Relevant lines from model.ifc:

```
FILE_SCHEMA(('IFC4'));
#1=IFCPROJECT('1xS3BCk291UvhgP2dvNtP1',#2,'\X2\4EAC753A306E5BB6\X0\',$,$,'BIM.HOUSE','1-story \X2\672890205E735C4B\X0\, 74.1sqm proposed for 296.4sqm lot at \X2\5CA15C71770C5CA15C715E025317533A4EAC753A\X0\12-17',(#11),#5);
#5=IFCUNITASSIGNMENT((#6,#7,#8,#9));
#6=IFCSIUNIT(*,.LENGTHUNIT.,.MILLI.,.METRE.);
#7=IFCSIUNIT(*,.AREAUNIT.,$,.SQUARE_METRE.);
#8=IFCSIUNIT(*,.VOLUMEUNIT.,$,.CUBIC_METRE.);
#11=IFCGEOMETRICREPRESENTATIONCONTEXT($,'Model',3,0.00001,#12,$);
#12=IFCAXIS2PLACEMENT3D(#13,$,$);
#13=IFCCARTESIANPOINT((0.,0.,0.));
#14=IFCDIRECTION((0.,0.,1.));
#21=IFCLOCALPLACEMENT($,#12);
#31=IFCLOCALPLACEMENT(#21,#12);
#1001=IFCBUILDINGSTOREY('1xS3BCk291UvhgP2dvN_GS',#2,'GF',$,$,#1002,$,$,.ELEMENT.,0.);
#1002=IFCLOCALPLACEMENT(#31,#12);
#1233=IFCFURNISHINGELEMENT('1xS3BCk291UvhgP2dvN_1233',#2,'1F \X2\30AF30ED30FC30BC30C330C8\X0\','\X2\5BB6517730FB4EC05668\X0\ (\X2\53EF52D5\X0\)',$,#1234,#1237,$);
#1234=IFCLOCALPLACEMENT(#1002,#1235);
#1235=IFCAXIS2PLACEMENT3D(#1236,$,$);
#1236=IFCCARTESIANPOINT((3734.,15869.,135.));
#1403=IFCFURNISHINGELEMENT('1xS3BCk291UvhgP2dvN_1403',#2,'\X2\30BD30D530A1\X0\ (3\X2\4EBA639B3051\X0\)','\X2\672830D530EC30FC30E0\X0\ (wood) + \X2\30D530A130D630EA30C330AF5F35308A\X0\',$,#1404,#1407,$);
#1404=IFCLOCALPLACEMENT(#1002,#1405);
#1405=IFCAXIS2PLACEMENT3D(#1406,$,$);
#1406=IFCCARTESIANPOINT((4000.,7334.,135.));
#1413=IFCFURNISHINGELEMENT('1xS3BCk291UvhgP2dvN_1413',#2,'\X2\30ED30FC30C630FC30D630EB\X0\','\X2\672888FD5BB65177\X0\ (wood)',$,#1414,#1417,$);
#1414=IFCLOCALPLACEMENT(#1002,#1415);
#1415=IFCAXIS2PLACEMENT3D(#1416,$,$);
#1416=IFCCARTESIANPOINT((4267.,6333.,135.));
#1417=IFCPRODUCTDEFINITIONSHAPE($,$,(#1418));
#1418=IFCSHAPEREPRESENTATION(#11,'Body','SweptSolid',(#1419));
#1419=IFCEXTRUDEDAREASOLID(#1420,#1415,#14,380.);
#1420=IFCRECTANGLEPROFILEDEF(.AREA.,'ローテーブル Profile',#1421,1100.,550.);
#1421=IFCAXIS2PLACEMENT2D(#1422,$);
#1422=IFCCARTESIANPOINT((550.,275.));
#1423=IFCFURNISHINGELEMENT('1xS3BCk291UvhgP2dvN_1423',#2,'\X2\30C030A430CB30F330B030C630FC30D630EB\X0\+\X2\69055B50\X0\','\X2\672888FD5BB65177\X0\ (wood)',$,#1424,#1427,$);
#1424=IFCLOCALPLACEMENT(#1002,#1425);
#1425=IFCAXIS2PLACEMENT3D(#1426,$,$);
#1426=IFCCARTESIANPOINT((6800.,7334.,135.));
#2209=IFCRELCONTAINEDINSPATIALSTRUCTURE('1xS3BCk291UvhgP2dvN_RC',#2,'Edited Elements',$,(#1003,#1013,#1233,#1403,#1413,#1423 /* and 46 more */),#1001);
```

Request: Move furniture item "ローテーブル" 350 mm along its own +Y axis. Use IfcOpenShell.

```python
import ifcopenshell
import ifcopenshell.api.geometry
import ifcopenshell.util.placement
import ifcopenshell.util.unit

model = ifcopenshell.open("model.ifc")
unit_scale = ifcopenshell.util.unit.calculate_unit_scale(model)

item = model.by_guid("1xS3BCk291UvhgP2dvN_1413")
matrix = ifcopenshell.util.placement.get_local_placement(item.ObjectPlacement)
matrix[:3, 3] += matrix[:3, 1] * 0.35 / unit_scale
ifcopenshell.api.geometry.edit_object_placement(model, product=item, matrix=matrix, is_si=False)

print(ifcopenshell.util.placement.get_local_placement(item.ObjectPlacement).round(3) + 0.0)

model.write("model_edited.ifc")
```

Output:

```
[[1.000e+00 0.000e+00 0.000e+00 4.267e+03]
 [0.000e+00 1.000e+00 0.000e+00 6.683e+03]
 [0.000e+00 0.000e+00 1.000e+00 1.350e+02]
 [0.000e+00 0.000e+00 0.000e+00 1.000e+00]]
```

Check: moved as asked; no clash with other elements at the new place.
